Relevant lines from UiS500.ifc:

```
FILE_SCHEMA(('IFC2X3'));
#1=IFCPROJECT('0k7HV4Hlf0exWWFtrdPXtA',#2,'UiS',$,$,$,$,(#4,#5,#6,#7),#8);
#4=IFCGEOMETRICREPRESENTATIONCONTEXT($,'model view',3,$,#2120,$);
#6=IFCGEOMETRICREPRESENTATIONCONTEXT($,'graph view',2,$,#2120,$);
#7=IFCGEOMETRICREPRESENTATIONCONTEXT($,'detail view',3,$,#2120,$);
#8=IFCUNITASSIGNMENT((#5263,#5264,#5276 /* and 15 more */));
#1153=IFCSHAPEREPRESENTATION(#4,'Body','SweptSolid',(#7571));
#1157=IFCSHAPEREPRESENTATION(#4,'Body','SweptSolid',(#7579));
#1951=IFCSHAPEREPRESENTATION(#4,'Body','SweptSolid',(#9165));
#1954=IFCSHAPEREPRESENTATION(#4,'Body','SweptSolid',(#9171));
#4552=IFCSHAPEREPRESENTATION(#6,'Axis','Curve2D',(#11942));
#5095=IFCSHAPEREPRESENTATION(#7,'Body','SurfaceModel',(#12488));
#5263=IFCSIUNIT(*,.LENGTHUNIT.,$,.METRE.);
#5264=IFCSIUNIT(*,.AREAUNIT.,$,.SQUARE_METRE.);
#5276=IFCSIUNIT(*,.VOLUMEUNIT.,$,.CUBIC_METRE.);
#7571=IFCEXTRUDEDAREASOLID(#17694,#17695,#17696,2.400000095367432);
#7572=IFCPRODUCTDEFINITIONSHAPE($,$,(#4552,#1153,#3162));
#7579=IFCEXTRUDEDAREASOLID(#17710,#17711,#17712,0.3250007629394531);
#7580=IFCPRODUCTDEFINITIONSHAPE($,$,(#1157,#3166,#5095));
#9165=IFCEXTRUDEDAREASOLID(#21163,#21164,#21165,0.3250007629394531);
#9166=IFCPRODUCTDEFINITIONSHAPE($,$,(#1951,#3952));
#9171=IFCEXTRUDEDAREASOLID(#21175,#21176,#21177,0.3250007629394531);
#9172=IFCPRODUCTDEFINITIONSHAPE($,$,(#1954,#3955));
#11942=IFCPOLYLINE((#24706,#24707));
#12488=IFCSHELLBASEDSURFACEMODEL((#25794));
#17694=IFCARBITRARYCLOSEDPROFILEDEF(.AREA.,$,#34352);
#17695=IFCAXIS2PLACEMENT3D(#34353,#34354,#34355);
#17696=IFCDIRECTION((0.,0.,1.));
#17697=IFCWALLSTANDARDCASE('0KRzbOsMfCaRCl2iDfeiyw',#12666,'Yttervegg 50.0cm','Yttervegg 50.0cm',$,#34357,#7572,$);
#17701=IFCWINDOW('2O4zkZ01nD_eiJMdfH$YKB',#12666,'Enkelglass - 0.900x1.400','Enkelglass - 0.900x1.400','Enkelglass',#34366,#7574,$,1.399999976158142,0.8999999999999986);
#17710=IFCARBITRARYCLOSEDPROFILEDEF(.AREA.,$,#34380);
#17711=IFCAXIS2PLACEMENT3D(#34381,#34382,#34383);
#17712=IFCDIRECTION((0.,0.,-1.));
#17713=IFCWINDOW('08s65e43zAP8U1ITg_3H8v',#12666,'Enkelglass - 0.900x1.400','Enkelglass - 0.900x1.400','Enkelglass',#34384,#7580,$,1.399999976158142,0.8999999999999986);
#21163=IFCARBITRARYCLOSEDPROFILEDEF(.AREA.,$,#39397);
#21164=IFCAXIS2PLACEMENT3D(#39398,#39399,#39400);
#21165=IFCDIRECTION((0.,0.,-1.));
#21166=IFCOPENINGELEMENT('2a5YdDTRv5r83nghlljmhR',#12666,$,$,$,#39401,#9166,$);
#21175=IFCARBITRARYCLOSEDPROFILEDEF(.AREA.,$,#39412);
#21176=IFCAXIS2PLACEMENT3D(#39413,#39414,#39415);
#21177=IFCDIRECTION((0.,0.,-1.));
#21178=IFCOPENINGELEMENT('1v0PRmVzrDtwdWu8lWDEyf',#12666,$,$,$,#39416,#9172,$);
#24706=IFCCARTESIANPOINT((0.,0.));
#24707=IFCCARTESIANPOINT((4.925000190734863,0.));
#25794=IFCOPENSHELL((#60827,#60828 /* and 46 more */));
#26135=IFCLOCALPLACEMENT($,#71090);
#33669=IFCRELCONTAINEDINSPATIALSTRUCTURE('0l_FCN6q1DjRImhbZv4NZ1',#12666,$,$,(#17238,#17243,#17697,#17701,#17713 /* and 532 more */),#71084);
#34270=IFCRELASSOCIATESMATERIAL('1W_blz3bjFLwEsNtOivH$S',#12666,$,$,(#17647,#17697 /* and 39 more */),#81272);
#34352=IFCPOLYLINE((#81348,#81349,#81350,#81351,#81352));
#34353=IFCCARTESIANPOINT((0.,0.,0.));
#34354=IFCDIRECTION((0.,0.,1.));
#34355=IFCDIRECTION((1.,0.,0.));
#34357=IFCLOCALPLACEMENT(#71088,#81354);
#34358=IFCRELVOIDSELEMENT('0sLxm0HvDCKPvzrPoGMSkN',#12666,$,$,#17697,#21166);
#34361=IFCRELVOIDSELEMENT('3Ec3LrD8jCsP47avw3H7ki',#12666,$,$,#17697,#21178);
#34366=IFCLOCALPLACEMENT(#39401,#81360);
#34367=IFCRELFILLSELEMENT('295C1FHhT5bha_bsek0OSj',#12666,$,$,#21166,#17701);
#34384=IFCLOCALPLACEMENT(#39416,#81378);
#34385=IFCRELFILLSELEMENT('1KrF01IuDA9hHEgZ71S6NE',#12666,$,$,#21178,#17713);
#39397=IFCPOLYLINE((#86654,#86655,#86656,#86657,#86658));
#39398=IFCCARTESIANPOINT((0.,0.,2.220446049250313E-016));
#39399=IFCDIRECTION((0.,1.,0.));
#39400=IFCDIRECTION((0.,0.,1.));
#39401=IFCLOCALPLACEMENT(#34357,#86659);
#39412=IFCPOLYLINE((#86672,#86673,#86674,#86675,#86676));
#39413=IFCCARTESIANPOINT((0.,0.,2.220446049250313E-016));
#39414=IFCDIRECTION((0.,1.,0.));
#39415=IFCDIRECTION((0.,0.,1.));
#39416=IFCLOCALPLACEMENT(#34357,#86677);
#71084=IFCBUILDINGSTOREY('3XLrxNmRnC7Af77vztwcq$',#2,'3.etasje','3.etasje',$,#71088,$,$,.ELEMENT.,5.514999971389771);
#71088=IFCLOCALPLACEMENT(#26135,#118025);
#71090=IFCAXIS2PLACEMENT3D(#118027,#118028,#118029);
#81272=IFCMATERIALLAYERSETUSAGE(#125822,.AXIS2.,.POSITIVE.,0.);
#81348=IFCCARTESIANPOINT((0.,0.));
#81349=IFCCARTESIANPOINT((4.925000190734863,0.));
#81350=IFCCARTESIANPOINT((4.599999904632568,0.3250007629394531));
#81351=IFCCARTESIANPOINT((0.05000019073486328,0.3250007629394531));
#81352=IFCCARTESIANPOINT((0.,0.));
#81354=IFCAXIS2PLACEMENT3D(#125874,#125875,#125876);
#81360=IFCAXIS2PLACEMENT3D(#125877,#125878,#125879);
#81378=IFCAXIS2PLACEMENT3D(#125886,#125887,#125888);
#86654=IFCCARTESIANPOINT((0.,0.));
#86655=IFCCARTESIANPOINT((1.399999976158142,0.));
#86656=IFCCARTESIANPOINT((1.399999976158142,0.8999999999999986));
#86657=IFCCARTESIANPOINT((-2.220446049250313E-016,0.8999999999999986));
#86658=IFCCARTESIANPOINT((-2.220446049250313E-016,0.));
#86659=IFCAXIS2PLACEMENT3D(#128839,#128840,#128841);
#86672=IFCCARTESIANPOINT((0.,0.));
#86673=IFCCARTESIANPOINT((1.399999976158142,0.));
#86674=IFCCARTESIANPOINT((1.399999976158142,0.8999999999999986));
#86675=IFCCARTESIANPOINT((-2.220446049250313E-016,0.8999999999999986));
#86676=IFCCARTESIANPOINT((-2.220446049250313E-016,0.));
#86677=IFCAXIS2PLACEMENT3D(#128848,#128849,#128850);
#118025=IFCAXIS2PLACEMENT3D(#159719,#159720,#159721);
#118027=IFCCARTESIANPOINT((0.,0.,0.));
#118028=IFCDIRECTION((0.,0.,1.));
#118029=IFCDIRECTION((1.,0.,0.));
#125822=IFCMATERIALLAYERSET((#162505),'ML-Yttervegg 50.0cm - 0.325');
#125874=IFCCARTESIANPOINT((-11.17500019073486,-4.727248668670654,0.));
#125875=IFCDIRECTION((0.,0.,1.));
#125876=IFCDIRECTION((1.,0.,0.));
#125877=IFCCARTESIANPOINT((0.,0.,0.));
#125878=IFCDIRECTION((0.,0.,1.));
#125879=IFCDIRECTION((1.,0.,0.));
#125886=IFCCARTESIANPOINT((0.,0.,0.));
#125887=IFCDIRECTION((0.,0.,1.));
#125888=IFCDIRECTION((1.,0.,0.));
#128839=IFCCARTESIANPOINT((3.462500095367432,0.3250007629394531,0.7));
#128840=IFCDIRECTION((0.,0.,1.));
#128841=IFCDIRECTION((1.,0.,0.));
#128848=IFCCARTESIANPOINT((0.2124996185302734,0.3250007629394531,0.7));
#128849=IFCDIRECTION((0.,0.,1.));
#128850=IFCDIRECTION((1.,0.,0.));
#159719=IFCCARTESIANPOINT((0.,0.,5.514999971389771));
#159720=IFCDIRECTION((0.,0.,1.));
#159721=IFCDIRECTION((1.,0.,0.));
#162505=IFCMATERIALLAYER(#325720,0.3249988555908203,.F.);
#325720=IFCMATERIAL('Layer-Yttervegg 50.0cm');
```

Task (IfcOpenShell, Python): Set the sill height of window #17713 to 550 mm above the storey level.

```python
import numpy as np
import ifcopenshell
import ifcopenshell.api.geometry
import ifcopenshell.geom
import ifcopenshell.util.element
import ifcopenshell.util.placement
import ifcopenshell.util.shape
import ifcopenshell.util.unit

model = ifcopenshell.open("UiS500.ifc")
unit_scale = ifcopenshell.util.unit.calculate_unit_scale(model)

window = model.by_guid("08s65e43zAP8U1ITg_3H8v")
opening = window.FillsVoids[0].RelatingOpeningElement
storey = ifcopenshell.util.element.get_container(window, ifc_class="IfcBuildingStorey")
level = ifcopenshell.util.placement.get_local_placement(storey.ObjectPlacement)[2, 3]

# The opening's origin need not be at the sill, so measure its lowest point.
shape = ifcopenshell.geom.create_shape(ifcopenshell.geom.settings(), opening)
bottom = ifcopenshell.util.shape.get_shape_bottom_elevation(shape, shape.geometry) / unit_scale
dz = level + 0.55 - bottom

shift = np.array([0.0, 0.0, dz])
# The window is placed relative to its opening, so it follows when the opening moves.
matrix = ifcopenshell.util.placement.get_local_placement(opening.ObjectPlacement)
matrix[:3, 3] += shift
ifcopenshell.api.geometry.edit_object_placement(
    model, product=opening, matrix=matrix, is_si=False, should_transform_children=True
)

print(f"moved by {dz * unit_scale:+.3f} m")

model.write("UiS500_v2.ifc")
```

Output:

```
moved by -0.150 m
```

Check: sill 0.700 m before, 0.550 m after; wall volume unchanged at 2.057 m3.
